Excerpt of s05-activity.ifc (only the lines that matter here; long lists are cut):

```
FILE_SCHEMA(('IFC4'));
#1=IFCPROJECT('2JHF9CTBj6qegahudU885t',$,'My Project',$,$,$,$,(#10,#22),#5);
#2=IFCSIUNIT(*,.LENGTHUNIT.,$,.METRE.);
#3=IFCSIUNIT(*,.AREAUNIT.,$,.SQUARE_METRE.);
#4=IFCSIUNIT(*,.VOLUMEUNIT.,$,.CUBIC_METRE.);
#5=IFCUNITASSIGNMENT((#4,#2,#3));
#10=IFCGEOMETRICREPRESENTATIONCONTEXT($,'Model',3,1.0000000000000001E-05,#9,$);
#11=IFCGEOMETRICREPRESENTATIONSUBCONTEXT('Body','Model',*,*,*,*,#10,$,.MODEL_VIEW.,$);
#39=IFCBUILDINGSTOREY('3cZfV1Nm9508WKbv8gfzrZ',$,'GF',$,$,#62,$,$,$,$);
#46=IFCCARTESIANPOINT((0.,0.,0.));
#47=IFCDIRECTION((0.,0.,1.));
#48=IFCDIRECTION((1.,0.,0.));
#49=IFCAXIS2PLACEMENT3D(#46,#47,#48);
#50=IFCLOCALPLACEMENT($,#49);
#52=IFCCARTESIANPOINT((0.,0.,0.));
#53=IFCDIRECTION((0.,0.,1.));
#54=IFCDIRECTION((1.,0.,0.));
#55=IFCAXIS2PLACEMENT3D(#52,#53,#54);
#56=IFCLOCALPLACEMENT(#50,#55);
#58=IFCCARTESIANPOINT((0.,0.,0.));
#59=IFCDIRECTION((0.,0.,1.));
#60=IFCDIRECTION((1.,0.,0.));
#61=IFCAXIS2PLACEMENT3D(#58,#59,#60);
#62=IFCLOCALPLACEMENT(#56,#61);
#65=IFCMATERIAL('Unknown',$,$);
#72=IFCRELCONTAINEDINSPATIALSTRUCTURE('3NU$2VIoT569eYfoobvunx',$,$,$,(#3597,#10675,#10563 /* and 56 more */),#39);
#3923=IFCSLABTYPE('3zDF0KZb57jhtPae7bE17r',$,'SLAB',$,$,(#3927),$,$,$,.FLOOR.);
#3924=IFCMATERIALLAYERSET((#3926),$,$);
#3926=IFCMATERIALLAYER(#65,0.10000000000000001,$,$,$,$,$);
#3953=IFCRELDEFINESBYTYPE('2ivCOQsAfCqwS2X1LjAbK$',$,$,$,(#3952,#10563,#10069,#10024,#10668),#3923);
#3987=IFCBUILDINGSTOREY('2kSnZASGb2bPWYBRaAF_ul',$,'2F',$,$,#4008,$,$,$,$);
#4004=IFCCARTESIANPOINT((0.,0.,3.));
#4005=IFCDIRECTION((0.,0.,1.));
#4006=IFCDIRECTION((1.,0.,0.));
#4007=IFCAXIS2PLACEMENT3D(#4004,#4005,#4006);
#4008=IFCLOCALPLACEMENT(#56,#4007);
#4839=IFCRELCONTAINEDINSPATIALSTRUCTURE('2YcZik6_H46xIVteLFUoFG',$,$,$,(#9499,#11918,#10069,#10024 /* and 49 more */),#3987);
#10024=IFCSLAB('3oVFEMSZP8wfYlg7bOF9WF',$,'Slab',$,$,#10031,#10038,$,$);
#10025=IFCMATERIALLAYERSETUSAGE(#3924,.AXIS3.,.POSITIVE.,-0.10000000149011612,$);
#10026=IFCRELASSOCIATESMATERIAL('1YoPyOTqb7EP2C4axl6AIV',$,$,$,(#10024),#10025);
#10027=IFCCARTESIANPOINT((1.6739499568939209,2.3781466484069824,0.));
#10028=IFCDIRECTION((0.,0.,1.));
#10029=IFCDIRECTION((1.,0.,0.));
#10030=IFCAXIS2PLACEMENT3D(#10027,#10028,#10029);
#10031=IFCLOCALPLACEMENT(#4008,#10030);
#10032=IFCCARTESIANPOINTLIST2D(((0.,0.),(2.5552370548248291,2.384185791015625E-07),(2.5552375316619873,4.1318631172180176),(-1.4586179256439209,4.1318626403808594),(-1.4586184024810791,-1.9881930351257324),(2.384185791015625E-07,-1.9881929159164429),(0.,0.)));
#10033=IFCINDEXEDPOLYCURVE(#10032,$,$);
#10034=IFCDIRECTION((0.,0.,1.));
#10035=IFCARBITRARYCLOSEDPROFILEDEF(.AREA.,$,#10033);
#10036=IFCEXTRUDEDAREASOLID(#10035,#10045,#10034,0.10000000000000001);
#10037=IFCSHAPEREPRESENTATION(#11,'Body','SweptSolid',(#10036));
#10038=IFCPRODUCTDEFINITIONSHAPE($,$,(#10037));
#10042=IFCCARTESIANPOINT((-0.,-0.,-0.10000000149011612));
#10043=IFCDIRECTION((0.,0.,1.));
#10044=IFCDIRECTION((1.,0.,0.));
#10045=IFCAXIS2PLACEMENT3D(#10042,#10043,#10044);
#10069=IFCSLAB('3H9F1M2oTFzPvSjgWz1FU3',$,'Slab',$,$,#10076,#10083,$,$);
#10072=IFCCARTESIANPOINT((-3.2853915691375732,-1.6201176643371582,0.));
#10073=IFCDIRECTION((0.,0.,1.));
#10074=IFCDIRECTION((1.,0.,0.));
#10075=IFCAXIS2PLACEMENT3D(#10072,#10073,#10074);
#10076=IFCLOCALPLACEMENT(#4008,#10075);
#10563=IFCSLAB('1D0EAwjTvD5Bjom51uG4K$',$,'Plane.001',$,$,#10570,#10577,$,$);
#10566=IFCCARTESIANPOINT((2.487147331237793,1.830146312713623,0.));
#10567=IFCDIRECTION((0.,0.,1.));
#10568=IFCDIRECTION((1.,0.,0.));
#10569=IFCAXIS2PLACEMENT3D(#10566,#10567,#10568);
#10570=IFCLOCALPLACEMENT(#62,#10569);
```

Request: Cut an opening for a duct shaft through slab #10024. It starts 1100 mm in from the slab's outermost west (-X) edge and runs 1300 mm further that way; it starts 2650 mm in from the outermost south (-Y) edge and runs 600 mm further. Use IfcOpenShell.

```python
import numpy as np
import ifcopenshell
import ifcopenshell.api.feature
import ifcopenshell.api.geometry
import ifcopenshell.api.root
import ifcopenshell.geom
import ifcopenshell.util.placement
import ifcopenshell.util.representation
import ifcopenshell.util.shape
import ifcopenshell.util.unit

model = ifcopenshell.open("s05-activity.ifc")
unit_scale = ifcopenshell.util.unit.calculate_unit_scale(model)
settings = ifcopenshell.geom.settings()


def volume(element):
    """Net volume in cubic metres, openings subtracted."""
    shape = ifcopenshell.geom.create_shape(settings, element)
    return ifcopenshell.util.shape.get_volume(shape.geometry)


slab = model.by_id(10024)
before = volume(slab)

# Extent in the slab's own axes, in metres. The edges named are its -X and -Y sides.
slab_shape = ifcopenshell.geom.create_shape(settings, slab)
vertices = ifcopenshell.util.shape.get_vertices(slab_shape.geometry)
x_min, y_min, bottom = vertices.min(axis=0)
top = vertices[:, 2].max()

opening = ifcopenshell.api.root.create_entity(model, ifc_class="IfcOpeningElement", name="Duct shaft opening", predefined_type="OPENING")
context = ifcopenshell.util.representation.get_context(model, "Model", "Body", "MODEL_VIEW")
width, depth = 1.3, 0.6
outline = [(0.0, 0.0), (width, 0.0), (width, depth), (0.0, depth), (0.0, 0.0)]
# Overshoot both faces by 50 mm so the cut is clean.
shape = ifcopenshell.api.geometry.add_slab_representation(
    model, context=context, depth=top - bottom + 0.1, polyline=outline
)
ifcopenshell.api.geometry.assign_representation(model, product=opening, representation=shape)

matrix = ifcopenshell.util.placement.get_local_placement(slab.ObjectPlacement)
matrix[:, 3] = matrix @ np.append(np.array([x_min + 1.1, y_min + 2.65, bottom - 0.05]) / unit_scale, 1.0)
ifcopenshell.api.geometry.edit_object_placement(model, product=opening, matrix=matrix, is_si=False)
ifcopenshell.api.feature.add_feature(model, feature=opening, element=slab)

after = volume(slab)

print(f"slab volume {before:.3f} -> {after:.3f} m3")

model.write("s05-activity_edited.ifc")
```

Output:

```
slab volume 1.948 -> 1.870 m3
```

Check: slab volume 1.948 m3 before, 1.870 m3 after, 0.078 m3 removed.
